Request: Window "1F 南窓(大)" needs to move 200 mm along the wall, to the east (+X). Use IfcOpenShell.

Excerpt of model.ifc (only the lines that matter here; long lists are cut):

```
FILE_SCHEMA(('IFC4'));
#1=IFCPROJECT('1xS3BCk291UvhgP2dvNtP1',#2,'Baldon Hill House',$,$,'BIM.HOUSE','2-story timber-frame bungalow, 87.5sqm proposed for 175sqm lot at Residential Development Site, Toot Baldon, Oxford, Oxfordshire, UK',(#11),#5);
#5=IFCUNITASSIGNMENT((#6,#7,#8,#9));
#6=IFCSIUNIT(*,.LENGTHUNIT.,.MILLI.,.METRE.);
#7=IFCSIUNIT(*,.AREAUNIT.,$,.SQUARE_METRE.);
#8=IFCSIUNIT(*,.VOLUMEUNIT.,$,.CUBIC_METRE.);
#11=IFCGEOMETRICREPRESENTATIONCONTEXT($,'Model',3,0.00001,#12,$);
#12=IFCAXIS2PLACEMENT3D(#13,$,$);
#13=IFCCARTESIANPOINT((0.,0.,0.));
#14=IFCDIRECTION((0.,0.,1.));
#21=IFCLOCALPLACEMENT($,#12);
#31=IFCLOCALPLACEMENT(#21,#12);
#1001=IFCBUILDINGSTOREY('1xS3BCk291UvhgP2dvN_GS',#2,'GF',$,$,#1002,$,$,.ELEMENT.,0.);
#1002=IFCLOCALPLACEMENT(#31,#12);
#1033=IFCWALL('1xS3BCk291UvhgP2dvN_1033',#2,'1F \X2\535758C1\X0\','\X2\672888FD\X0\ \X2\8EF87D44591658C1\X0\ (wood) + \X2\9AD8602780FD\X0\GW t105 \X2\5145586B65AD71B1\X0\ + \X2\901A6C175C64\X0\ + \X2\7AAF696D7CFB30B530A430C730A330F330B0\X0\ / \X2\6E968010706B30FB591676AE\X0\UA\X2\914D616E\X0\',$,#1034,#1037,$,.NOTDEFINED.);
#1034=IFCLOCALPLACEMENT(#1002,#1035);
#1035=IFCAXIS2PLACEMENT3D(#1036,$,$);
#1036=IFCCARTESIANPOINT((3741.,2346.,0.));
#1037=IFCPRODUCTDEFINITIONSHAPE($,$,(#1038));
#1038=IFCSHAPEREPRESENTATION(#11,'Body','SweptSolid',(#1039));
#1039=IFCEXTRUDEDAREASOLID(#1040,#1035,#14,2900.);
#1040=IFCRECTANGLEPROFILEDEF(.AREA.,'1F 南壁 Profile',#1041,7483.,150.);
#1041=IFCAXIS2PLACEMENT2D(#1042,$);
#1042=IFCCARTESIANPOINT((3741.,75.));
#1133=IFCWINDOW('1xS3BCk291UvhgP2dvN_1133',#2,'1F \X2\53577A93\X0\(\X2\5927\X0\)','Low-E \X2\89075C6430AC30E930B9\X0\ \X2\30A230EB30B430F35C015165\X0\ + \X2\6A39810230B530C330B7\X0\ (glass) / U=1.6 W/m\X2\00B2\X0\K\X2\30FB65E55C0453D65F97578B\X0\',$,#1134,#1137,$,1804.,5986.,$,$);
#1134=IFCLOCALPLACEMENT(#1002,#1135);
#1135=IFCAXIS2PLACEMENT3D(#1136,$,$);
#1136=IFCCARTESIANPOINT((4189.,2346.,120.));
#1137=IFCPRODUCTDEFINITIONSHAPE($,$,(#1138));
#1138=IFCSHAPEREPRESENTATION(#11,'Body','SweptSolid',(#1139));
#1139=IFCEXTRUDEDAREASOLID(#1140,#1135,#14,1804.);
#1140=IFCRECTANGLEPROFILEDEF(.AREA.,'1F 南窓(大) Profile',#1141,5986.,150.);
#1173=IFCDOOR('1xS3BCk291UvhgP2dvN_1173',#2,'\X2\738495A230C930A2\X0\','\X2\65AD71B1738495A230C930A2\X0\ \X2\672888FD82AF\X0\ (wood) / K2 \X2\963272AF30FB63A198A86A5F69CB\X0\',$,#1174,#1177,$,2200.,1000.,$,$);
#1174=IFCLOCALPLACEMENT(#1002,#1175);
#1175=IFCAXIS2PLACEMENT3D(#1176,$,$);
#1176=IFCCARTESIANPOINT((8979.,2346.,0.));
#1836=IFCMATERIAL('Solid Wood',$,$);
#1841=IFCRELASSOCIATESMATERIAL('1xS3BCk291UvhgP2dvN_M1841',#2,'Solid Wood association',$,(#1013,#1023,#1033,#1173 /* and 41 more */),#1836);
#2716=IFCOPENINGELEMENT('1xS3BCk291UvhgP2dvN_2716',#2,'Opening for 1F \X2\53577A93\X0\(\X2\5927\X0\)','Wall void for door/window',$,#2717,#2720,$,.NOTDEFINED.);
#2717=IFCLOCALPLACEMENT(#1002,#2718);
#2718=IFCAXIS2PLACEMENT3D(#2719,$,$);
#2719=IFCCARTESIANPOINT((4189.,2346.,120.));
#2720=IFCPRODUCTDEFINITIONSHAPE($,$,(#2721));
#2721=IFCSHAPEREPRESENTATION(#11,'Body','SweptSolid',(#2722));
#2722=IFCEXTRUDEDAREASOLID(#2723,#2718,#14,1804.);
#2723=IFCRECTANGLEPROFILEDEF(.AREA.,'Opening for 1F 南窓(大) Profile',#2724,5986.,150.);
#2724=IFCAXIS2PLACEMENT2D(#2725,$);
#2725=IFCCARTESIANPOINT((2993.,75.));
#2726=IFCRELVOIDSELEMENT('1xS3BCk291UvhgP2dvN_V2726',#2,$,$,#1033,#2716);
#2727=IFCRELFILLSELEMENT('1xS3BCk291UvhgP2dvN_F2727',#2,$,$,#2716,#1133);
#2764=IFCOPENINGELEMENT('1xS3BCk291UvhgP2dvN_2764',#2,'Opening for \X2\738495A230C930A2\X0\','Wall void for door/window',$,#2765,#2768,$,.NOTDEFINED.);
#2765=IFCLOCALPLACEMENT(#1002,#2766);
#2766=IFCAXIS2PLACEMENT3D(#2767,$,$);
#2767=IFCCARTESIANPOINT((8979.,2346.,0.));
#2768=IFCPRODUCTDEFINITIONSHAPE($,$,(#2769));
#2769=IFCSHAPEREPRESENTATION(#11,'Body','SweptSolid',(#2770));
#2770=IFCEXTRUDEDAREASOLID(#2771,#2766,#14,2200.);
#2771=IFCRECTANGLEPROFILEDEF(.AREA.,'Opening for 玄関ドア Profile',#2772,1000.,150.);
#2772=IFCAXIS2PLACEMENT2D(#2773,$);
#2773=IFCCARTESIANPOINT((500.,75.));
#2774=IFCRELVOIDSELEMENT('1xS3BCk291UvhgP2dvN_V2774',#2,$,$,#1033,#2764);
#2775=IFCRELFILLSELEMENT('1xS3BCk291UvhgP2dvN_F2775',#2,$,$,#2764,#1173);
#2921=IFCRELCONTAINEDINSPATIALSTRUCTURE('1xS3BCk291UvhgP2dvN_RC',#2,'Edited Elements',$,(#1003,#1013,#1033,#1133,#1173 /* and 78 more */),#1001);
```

```python
import ifcopenshell
import ifcopenshell.api.geometry
import ifcopenshell.util.placement
import ifcopenshell.util.unit

model = ifcopenshell.open("model.ifc")
unit_scale = ifcopenshell.util.unit.calculate_unit_scale(model)

window = model.by_id(1133)
opening = window.FillsVoids[0].RelatingOpeningElement
wall = opening.VoidsElements[0].RelatingBuildingElement

wall_matrix = ifcopenshell.util.placement.get_local_placement(wall.ObjectPlacement)
shift = wall_matrix[:3, 0] * 0.2 / unit_scale
before = ifcopenshell.util.placement.get_local_placement(window.ObjectPlacement)[:3, 3].copy()

# The window is not placed relative to its opening, so move both.
for product in (opening, window):
    matrix = ifcopenshell.util.placement.get_local_placement(product.ObjectPlacement)
    matrix[:3, 3] += shift
    ifcopenshell.api.geometry.edit_object_placement(model, product=product, matrix=matrix, is_si=False)

after = ifcopenshell.util.placement.get_local_placement(window.ObjectPlacement)[:3, 3]
print("window moved by", (after - before).round(3) + 0.0)

model.write("model-out.ifc")
```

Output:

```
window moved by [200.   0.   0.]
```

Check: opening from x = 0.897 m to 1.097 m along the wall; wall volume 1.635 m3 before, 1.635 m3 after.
